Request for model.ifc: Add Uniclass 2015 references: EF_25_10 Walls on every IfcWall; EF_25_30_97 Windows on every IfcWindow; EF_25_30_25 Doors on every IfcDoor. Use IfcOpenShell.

First a look at what the model holds.

```python
import ifcopenshell

model = ifcopenshell.open("model.ifc")
print(model.schema)
print("classifications:", [c.Name for c in model.by_type("IfcClassification")])
for ifc_class in ("IfcDoor", "IfcRoof", "IfcStair", "IfcWall", "IfcWindow"):
    print(ifc_class, len(model.by_type(ifc_class)))
```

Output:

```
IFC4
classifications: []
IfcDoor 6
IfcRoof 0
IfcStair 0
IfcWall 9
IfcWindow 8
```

```python
import ifcopenshell
import ifcopenshell.api.classification

model = ifcopenshell.open("model.ifc")

system = ifcopenshell.api.classification.add_classification(model, classification="Uniclass 2015")

codes = {
    "IfcWall": ("EF_25_10", "Walls"),
    "IfcWindow": ("EF_25_30_97", "Windows"),
    "IfcDoor": ("EF_25_30_25", "Doors"),
}
for ifc_class, (code, name) in codes.items():
    products = model.by_type(ifc_class)
    ifcopenshell.api.classification.add_reference(
        model, products=products, classification=system, identification=code, name=name
    )
    print(code, len(products))

model.write("model_updated.ifc")
```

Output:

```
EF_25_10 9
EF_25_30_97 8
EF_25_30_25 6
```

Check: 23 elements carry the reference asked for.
